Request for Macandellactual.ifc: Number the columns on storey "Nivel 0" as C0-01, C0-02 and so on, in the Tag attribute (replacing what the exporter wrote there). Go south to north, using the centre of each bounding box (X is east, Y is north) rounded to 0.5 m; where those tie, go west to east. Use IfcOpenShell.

First a look at what the model holds.

```python
import ifcopenshell
import ifcopenshell.util.element
import ifcopenshell.util.placement

model = ifcopenshell.open("Macandellactual.ifc")
print(model.schema)
storey = next(s for s in model.by_type("IfcBuildingStorey") if s.Name == "Nivel 0")
columns = [e for e in ifcopenshell.util.element.get_decomposition(storey) if e.is_a("IfcColumn")]
for e in sorted(columns, key=lambda e: e.id()):
    origin = ifcopenshell.util.placement.get_local_placement(e.ObjectPlacement)[:3, 3]
    print(e.id(), e.Tag, e.Name, origin.round(2) + 0.0, sep=" | ")
```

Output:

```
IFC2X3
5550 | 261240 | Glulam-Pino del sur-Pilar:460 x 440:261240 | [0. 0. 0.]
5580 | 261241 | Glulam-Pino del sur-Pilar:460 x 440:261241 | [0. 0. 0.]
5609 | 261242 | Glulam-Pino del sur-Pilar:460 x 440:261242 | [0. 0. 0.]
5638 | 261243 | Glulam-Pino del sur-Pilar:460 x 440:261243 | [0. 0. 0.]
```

```python
import ifcopenshell
import ifcopenshell.geom
import ifcopenshell.util.element
import ifcopenshell.util.shape

model = ifcopenshell.open("Macandellactual.ifc")
settings = ifcopenshell.geom.settings()
settings.set("use-world-coords", True)


def centre(element):
    shape = ifcopenshell.geom.create_shape(settings, element)
    return ifcopenshell.util.shape.get_bbox_centroid(shape.geometry)


storey = next(s for s in model.by_type("IfcBuildingStorey") if s.Name == "Nivel 0")
columns = [e for e in ifcopenshell.util.element.get_decomposition(storey) if e.is_a("IfcColumn")]

# Insertion points can sit at a corner or the storey origin, so sort by the geometry (in metres).
centres = {e: centre(e) for e in columns}
columns.sort(key=lambda e: (round(centres[e][1] / 0.5), centres[e][0]))

for i, e in enumerate(columns, start=1):
    number = f"C0-{i:02d}"
    e.Tag = number
    print(e.id(), number)

model.write("Macandellactual_v2.ifc")
```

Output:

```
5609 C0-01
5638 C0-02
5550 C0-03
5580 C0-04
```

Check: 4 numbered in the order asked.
